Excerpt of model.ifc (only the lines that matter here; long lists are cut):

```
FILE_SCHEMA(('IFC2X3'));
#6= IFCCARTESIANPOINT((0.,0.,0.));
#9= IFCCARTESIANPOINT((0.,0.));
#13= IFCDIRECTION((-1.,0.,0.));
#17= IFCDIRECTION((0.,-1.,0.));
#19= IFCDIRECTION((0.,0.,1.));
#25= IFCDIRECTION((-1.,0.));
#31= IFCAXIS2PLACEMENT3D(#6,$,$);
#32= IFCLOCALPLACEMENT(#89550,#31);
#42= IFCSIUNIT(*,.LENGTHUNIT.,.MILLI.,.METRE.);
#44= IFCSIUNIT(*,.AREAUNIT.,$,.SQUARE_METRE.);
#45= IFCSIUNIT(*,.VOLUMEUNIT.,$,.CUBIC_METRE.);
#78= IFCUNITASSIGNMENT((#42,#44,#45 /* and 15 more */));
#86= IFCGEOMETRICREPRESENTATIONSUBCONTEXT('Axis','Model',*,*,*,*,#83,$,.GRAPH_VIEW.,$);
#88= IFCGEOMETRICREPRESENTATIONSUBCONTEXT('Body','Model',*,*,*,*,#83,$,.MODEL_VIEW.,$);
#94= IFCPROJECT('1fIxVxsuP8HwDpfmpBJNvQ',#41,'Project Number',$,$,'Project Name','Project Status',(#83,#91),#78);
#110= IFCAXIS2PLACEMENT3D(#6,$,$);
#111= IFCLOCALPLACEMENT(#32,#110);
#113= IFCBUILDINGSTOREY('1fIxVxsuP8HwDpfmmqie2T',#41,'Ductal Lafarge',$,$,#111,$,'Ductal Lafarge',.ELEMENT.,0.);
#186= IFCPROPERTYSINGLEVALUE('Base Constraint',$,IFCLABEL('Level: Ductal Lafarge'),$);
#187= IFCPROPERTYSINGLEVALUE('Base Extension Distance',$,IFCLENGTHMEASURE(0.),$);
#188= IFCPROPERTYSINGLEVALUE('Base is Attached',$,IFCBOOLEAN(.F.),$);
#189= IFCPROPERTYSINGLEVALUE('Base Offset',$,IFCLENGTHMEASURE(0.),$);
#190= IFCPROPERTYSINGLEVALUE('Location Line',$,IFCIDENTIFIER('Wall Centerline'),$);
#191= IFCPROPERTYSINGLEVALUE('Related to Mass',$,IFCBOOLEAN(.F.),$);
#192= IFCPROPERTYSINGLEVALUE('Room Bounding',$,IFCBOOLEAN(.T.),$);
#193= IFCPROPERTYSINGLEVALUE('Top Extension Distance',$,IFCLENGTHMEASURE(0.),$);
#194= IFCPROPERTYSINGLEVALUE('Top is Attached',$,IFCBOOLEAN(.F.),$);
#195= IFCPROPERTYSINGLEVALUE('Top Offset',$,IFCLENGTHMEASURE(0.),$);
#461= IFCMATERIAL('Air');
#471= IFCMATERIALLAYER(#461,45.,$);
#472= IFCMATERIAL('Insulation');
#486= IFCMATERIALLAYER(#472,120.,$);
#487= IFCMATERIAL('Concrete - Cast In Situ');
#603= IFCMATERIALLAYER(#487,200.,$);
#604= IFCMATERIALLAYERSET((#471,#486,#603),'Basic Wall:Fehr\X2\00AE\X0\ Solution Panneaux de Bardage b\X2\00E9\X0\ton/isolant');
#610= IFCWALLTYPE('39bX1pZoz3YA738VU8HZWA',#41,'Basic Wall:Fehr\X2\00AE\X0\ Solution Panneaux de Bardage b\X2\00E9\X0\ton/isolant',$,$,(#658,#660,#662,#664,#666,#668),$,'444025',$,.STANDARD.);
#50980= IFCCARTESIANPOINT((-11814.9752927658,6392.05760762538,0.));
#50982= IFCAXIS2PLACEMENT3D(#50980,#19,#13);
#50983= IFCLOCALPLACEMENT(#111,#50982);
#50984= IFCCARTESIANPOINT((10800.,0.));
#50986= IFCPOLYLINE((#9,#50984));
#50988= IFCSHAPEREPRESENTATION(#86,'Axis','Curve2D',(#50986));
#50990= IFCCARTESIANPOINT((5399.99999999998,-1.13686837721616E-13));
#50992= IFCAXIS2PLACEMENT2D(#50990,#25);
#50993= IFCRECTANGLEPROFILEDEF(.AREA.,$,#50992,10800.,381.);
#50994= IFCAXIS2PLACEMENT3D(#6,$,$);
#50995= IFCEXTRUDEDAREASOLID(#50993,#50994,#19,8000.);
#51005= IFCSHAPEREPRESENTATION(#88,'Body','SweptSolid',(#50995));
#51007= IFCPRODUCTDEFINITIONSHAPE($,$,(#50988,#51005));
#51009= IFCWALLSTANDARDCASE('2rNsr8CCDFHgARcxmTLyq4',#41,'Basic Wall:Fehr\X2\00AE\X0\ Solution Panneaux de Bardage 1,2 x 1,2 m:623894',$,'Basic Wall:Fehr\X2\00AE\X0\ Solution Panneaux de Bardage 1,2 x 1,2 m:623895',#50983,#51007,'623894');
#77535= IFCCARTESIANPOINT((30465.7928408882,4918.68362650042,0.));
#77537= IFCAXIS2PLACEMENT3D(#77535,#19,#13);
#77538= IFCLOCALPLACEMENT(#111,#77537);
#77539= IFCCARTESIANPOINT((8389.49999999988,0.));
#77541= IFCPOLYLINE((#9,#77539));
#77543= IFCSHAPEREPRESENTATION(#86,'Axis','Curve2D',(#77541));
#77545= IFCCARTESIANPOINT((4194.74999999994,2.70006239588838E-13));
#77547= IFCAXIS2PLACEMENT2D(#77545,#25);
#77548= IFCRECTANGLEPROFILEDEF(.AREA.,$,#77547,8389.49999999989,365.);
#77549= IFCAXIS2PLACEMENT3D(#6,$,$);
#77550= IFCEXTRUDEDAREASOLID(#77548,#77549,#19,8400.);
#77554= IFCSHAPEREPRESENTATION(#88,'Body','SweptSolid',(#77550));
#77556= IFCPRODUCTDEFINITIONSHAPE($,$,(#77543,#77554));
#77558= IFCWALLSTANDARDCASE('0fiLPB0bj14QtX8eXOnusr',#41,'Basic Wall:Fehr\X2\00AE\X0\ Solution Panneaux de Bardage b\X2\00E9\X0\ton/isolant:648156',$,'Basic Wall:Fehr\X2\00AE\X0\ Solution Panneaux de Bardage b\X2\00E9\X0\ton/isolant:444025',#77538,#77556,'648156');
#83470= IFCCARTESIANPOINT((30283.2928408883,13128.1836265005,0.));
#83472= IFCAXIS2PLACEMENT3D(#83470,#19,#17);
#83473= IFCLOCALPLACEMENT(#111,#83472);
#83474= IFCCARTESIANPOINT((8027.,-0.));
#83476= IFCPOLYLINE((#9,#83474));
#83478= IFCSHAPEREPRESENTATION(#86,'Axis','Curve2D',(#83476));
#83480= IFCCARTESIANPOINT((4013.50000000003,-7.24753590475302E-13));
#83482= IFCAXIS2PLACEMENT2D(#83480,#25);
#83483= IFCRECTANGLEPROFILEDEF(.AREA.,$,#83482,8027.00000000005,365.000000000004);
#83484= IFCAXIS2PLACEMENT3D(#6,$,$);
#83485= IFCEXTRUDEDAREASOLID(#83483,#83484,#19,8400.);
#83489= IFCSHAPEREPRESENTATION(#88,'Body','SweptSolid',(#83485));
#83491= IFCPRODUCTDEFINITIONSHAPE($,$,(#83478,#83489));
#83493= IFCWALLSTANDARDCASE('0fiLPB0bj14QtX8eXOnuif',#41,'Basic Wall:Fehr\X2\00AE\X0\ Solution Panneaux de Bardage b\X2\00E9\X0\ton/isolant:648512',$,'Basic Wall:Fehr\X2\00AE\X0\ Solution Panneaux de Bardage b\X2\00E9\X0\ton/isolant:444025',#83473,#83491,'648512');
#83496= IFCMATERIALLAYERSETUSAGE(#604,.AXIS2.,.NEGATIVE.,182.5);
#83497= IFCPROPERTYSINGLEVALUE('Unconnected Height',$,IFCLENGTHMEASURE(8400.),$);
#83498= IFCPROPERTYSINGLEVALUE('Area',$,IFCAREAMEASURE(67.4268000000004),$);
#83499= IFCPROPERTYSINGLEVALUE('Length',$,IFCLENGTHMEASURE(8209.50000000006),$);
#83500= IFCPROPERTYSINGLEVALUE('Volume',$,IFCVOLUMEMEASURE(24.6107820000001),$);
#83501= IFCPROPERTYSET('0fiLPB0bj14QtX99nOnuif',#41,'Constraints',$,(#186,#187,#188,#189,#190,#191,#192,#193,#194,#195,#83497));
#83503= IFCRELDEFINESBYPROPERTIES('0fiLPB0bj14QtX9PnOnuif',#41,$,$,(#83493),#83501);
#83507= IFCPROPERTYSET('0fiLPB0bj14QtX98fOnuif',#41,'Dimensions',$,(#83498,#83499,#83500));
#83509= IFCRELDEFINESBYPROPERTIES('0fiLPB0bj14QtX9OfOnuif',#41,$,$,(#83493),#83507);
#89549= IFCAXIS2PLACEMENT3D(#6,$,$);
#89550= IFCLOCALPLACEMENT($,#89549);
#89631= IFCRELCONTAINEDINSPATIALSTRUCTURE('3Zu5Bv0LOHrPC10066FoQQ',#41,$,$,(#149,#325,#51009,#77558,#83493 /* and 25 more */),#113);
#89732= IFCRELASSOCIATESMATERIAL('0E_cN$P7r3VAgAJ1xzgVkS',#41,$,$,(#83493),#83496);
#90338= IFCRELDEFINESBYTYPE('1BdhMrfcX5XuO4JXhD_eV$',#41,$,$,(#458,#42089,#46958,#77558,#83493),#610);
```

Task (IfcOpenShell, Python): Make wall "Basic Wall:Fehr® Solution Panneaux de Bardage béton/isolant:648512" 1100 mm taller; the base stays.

```python
import ifcopenshell
import ifcopenshell.api.pset
import ifcopenshell.geom
import ifcopenshell.util.element
import ifcopenshell.util.representation
import ifcopenshell.util.shape
import ifcopenshell.util.unit

model = ifcopenshell.open("model.ifc")
area_scale = ifcopenshell.util.unit.calculate_unit_scale(model, "AREAUNIT")
volume_scale = ifcopenshell.util.unit.calculate_unit_scale(model, "VOLUMEUNIT")
settings = ifcopenshell.geom.settings()


def volume(element):
    """Net volume in cubic metres, openings subtracted."""
    shape = ifcopenshell.geom.create_shape(settings, element)
    return ifcopenshell.util.shape.get_volume(shape.geometry)


wall = model.by_guid("0fiLPB0bj14QtX8eXOnuif")
before = volume(wall)

body = ifcopenshell.util.representation.get_representation(wall, "Model", "Body")
solid = body.Items[0]
old_height = solid.Depth
solid.Depth += 1100.0
after = volume(wall)
thickness = 0.365  # wall thickness in metres

# Update the stored height, areas and volumes.
pset = model.by_id(ifcopenshell.util.element.get_pset(wall, "Constraints", should_inherit=False)["id"])
ifcopenshell.api.pset.edit_pset(model, pset=pset, properties={
    "Unconnected Height": model.create_entity("IfcLengthMeasure", solid.Depth),
})
pset = model.by_id(ifcopenshell.util.element.get_pset(wall, "Dimensions", should_inherit=False)["id"])
ifcopenshell.api.pset.edit_pset(model, pset=pset, properties={
    "Area": model.create_entity("IfcAreaMeasure", after / thickness / area_scale),
    "Volume": model.create_entity("IfcVolumeMeasure", after / volume_scale),
})

print(f"height {old_height:g} -> {solid.Depth:g}, volume {before:.3f} -> {after:.3f} m3")

model.write("model_v2.ifc")
```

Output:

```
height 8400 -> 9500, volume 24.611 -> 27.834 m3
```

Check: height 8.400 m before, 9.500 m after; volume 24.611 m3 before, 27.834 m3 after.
